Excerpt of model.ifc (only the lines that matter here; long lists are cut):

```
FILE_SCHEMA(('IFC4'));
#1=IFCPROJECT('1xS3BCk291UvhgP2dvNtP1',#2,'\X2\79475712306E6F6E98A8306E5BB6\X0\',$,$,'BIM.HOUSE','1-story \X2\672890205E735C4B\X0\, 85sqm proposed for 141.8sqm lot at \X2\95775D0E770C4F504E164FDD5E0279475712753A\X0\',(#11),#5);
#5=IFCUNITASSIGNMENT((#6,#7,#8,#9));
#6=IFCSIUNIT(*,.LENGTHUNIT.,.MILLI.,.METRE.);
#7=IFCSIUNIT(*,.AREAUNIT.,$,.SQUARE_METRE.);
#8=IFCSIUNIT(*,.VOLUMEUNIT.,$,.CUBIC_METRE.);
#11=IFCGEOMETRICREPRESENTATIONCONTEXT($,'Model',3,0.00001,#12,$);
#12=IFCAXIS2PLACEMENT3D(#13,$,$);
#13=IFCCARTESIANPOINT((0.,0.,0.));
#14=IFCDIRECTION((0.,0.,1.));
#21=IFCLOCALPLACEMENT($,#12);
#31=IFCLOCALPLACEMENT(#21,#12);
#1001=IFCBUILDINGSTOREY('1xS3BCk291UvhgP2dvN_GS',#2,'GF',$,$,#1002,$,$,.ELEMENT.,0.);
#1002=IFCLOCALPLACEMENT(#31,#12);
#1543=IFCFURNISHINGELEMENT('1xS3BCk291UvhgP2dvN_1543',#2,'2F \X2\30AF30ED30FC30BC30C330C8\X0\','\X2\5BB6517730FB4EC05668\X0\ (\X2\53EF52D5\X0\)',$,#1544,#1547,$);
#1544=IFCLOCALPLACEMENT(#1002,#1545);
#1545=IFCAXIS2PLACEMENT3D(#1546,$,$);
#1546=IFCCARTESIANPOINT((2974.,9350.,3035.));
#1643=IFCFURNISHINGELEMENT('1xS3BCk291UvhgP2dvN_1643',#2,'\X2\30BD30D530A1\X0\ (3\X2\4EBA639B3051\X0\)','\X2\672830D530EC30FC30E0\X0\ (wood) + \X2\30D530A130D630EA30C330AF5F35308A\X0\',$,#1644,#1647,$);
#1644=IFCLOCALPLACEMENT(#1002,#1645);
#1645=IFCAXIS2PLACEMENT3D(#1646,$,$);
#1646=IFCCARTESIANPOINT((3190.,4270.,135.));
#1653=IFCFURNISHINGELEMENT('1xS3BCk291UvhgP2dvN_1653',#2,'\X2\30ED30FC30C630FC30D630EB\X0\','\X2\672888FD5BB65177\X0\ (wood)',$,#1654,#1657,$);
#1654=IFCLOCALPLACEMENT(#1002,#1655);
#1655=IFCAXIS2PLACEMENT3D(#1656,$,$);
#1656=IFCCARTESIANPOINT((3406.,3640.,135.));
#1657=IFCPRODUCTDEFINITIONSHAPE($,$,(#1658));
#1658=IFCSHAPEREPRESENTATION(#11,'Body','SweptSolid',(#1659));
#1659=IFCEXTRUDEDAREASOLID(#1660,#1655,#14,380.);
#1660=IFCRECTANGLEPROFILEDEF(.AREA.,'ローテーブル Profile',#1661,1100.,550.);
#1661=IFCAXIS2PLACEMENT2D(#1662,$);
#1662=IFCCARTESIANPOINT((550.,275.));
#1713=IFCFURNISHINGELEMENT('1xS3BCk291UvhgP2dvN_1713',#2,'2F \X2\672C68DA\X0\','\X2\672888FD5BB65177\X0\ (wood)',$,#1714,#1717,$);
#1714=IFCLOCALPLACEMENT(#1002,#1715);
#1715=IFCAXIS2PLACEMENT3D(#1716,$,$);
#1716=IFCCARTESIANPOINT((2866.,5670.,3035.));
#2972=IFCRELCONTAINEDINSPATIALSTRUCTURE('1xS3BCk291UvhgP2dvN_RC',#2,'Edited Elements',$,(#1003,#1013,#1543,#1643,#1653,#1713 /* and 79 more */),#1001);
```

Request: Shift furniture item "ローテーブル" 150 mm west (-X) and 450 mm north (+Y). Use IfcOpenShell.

```python
import ifcopenshell
import ifcopenshell.api.geometry
import ifcopenshell.util.placement

model = ifcopenshell.open("model.ifc")

item = model.by_id(1653)
matrix = ifcopenshell.util.placement.get_local_placement(item.ObjectPlacement)
matrix[0, 3] -= 150.0
matrix[1, 3] += 450.0
ifcopenshell.api.geometry.edit_object_placement(model, product=item, matrix=matrix, is_si=False)

print(ifcopenshell.util.placement.get_local_placement(item.ObjectPlacement).round(3) + 0.0)

model.write("model_v2.ifc")
```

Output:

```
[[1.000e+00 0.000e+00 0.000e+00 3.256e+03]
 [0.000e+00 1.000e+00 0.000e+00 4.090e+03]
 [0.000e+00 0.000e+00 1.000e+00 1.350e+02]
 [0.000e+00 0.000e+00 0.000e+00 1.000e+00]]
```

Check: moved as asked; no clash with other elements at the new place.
